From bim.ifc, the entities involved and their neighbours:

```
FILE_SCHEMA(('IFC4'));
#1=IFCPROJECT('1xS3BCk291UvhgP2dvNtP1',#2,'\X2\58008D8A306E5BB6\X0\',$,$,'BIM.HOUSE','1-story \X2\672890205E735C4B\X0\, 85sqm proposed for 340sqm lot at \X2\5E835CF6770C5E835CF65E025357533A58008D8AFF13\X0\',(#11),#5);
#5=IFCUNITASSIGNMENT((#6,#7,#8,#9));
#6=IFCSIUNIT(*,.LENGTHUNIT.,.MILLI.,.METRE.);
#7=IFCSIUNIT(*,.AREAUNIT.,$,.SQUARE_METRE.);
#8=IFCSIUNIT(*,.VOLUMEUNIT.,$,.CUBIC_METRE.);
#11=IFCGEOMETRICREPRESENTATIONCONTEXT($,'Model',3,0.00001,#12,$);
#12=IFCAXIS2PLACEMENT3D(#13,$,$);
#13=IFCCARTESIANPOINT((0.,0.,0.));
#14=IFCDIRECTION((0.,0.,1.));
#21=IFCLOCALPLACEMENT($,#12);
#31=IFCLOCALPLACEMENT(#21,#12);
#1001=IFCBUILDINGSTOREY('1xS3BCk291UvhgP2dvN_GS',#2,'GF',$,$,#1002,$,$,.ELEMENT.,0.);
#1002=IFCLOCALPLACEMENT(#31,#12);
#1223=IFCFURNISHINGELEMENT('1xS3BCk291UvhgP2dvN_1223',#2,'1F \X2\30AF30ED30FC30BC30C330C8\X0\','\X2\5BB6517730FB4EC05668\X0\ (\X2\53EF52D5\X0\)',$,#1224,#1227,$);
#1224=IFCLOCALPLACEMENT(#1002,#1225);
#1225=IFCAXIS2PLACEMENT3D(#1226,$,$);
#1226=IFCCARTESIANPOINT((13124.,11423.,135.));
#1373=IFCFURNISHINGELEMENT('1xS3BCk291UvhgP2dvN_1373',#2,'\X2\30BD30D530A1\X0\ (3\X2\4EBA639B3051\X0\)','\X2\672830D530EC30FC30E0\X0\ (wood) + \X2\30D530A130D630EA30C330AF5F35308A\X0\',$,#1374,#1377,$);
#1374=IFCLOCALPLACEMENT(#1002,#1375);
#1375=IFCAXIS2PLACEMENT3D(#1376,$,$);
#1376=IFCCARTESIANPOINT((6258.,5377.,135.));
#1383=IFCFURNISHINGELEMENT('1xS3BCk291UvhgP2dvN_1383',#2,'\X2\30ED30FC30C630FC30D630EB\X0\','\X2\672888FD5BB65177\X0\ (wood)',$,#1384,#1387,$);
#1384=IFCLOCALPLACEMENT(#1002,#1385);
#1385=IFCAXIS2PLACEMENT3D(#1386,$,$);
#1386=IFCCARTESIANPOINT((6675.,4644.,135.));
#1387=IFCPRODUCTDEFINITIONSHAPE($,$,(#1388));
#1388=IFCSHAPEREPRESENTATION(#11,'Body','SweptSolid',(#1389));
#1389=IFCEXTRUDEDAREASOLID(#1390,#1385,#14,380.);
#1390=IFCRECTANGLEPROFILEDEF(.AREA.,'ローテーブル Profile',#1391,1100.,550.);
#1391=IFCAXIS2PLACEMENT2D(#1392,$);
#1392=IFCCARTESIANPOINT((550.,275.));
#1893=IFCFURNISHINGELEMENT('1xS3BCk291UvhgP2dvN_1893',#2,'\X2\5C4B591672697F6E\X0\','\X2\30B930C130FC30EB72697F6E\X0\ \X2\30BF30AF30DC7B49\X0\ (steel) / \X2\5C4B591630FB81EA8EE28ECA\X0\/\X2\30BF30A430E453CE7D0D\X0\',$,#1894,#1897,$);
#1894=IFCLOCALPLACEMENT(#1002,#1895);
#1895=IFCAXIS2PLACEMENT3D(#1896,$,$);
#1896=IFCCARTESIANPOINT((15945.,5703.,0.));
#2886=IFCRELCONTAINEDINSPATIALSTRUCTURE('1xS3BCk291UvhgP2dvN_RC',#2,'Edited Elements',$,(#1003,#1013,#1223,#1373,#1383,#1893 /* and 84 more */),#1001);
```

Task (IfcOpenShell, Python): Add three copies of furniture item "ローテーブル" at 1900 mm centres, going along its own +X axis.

```python
import ifcopenshell
import ifcopenshell.api.geometry
import ifcopenshell.api.root
import ifcopenshell.util.element
import ifcopenshell.util.placement
import ifcopenshell.util.unit

model = ifcopenshell.open("bim.ifc")
unit_scale = ifcopenshell.util.unit.calculate_unit_scale(model)


def reuse_history(source, copy):
    """copy_class also copies each property set's owner history, people and application; keep the originals."""
    for rel in copy.IsDefinedBy:
        if rel.is_a("IfcRelDefinesByProperties") and (history := rel.RelatingPropertyDefinition.OwnerHistory):
            rel.RelatingPropertyDefinition.OwnerHistory = source.OwnerHistory
            ifcopenshell.util.element.remove_deep2(model, history)


source = model.by_guid("1xS3BCk291UvhgP2dvN_1383")
base = ifcopenshell.util.placement.get_local_placement(source.ObjectPlacement)
step = base[:3, 0] * 1.9 / unit_scale

for i in range(1, 4):
    copy = ifcopenshell.api.root.copy_class(model, product=source)
    copy.Representation = ifcopenshell.util.element.copy_deep(
        model, source.Representation, exclude=["IfcGeometricRepresentationContext", "IfcRepresentationMap"]
    )
    reuse_history(source, copy)
    matrix = base.copy()
    matrix[:3, 3] += i * step
    print("added at", matrix[:3, 3].round(3) + 0.0)
    ifcopenshell.api.geometry.edit_object_placement(model, product=copy, matrix=matrix, is_si=False)

model.write("bim_v2.ifc")
```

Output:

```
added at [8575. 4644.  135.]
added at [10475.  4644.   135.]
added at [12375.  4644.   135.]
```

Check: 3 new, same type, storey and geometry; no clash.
